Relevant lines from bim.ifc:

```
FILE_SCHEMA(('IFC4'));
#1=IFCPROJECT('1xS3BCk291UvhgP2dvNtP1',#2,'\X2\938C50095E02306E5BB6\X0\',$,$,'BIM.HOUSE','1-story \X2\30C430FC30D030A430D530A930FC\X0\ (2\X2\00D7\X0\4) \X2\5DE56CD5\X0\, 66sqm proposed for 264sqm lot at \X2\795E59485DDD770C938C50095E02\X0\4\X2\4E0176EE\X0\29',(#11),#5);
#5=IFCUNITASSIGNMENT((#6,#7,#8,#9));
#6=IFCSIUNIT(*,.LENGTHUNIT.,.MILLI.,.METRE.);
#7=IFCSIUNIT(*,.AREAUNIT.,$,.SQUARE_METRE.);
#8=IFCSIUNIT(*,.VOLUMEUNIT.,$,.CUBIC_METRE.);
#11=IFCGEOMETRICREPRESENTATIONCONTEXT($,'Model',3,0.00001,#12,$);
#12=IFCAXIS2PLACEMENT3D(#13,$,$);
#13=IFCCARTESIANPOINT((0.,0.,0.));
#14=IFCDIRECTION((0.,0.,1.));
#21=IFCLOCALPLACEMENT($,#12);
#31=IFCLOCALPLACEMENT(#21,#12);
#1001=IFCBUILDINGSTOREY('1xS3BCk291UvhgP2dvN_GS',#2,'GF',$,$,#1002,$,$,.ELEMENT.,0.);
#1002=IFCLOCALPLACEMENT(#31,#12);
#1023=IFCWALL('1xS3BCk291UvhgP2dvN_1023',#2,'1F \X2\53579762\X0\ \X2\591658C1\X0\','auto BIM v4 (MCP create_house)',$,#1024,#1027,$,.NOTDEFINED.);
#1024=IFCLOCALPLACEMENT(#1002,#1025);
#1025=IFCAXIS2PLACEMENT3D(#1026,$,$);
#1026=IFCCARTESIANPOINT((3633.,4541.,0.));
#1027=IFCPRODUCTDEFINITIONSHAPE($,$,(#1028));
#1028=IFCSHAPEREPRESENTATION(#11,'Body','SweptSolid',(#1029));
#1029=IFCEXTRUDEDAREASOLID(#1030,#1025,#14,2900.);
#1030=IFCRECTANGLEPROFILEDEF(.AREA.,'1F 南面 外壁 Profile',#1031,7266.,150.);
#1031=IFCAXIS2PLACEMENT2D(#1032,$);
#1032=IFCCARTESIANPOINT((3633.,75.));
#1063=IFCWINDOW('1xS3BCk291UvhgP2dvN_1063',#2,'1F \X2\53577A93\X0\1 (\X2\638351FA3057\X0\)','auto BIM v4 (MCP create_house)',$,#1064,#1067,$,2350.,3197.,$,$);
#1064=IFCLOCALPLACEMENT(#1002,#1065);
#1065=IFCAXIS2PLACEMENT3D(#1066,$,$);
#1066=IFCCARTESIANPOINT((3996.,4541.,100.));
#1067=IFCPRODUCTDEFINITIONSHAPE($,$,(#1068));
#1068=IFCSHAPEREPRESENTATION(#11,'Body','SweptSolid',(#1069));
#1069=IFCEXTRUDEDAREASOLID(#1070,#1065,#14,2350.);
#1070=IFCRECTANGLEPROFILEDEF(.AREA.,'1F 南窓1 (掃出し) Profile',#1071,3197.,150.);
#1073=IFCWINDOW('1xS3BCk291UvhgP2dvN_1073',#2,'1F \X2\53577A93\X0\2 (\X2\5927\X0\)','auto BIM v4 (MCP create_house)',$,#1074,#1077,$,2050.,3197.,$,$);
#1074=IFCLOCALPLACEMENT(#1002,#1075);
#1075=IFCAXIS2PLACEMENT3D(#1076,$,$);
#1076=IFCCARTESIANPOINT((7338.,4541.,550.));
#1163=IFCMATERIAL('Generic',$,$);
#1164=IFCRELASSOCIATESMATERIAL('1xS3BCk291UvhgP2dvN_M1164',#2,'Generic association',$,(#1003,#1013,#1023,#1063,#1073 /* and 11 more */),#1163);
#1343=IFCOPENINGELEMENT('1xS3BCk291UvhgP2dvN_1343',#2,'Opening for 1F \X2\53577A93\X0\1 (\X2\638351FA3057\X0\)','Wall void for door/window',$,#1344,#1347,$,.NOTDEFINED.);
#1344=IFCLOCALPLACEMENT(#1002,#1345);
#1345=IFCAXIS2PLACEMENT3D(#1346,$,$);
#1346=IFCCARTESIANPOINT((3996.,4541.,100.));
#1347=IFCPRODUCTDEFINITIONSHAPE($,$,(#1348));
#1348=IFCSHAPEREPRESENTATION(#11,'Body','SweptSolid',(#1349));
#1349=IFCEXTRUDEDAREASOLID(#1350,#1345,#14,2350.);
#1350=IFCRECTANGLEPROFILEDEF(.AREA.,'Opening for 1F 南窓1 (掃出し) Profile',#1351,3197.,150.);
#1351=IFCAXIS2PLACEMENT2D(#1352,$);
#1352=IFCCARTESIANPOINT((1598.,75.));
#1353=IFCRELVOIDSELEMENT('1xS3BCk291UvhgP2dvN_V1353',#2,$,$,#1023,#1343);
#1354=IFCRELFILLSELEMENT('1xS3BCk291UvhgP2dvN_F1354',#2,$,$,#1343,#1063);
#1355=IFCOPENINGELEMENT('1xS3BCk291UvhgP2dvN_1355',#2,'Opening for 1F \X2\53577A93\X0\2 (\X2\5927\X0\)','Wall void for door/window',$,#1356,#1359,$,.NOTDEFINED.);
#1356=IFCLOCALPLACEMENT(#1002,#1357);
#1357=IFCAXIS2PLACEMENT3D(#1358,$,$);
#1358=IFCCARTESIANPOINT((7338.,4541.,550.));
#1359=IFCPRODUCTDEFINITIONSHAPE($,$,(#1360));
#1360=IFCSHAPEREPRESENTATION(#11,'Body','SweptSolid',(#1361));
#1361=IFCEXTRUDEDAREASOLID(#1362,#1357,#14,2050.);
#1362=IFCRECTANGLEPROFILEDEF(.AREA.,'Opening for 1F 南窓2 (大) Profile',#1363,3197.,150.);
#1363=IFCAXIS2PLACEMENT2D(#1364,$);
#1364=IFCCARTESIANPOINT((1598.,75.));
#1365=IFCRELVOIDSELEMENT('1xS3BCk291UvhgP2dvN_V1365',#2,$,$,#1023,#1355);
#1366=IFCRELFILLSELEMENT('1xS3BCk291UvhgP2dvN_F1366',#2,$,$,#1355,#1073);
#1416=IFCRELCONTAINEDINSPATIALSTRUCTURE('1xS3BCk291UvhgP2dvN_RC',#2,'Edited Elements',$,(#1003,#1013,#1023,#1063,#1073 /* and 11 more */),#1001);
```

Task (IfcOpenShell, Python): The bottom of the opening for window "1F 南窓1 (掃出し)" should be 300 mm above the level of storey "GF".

```python
import numpy as np
import ifcopenshell
import ifcopenshell.api.geometry
import ifcopenshell.geom
import ifcopenshell.util.element
import ifcopenshell.util.placement
import ifcopenshell.util.shape
import ifcopenshell.util.unit

model = ifcopenshell.open("bim.ifc")
unit_scale = ifcopenshell.util.unit.calculate_unit_scale(model)

window = model.by_id(1063)
opening = window.FillsVoids[0].RelatingOpeningElement
storey = ifcopenshell.util.element.get_container(window, ifc_class="IfcBuildingStorey")
level = ifcopenshell.util.placement.get_local_placement(storey.ObjectPlacement)[2, 3]

# The opening's origin need not be at the sill, so measure its lowest point.
shape = ifcopenshell.geom.create_shape(ifcopenshell.geom.settings(), opening)
bottom = ifcopenshell.util.shape.get_shape_bottom_elevation(shape, shape.geometry) / unit_scale
dz = level + 0.3 / unit_scale - bottom

shift = np.array([0.0, 0.0, dz])
# The window is not placed relative to its opening, so move both.
for product in (opening, window):
    matrix = ifcopenshell.util.placement.get_local_placement(product.ObjectPlacement)
    matrix[:3, 3] += shift
    ifcopenshell.api.geometry.edit_object_placement(model, product=product, matrix=matrix, is_si=False)

print(f"moved by {dz * unit_scale:+.3f} m")

model.write("bim_rev.ifc")
```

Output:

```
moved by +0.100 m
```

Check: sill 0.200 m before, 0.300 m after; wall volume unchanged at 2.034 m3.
